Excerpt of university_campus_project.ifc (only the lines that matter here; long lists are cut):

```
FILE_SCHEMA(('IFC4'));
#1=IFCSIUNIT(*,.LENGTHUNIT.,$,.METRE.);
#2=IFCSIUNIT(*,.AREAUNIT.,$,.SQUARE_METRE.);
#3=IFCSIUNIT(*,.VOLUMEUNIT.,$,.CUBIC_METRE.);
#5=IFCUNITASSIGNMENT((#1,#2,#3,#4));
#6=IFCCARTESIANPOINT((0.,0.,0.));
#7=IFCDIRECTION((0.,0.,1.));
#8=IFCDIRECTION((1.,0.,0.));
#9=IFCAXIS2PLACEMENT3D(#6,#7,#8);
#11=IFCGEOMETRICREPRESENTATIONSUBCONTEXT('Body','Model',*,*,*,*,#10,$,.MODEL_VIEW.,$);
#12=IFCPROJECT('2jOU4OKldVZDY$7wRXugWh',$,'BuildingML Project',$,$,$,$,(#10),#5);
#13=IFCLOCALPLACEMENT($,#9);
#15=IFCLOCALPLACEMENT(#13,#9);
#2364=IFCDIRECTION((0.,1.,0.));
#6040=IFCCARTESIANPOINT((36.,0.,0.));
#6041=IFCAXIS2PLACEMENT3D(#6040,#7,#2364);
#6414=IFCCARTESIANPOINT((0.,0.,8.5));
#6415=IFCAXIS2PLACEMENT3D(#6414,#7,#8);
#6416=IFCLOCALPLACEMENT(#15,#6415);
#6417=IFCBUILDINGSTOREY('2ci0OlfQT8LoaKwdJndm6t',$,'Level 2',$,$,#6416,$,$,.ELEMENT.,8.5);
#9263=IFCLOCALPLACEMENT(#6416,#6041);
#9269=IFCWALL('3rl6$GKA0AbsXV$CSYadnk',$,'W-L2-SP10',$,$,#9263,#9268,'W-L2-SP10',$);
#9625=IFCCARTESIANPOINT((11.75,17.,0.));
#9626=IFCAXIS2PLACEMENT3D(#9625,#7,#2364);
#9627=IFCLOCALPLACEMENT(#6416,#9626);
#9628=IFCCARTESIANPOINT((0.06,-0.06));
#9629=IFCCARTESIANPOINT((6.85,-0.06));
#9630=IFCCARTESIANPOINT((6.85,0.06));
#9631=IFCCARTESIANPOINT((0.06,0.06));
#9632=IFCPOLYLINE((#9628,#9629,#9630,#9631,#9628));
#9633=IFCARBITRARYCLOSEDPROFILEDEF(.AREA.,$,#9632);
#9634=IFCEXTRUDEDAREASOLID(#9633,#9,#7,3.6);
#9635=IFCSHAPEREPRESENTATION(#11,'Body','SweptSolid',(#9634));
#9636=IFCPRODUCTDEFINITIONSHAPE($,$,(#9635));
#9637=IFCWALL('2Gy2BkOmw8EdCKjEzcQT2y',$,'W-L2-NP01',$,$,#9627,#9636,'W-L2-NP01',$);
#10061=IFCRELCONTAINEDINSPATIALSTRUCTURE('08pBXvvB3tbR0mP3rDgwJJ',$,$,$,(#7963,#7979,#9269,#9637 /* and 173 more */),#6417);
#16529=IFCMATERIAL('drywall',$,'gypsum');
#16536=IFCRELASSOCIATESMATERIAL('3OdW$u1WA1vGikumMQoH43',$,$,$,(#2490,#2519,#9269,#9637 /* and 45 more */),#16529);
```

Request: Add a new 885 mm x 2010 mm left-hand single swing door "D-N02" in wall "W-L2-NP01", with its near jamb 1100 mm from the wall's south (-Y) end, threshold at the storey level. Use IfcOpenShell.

```python
import numpy as np
import ifcopenshell
import ifcopenshell.api.feature
import ifcopenshell.api.geometry
import ifcopenshell.api.root
import ifcopenshell.api.spatial
import ifcopenshell.geom
import ifcopenshell.util.element
import ifcopenshell.util.placement
import ifcopenshell.util.representation
import ifcopenshell.util.shape
import ifcopenshell.util.unit

model = ifcopenshell.open("university_campus_project.ifc")
unit_scale = ifcopenshell.util.unit.calculate_unit_scale(model)
settings = ifcopenshell.geom.settings()


def volume(element):
    """Net volume in cubic metres, openings subtracted."""
    shape = ifcopenshell.geom.create_shape(settings, element)
    return ifcopenshell.util.shape.get_volume(shape.geometry)


wall = model.by_id(9637)
storey = ifcopenshell.util.element.get_container(wall, ifc_class="IfcBuildingStorey")
context = ifcopenshell.util.representation.get_context(model, "Model", "Body", "MODEL_VIEW")
before = volume(wall)

width, height, from_end, sill = 0.885, 2.01, 1.1, 0.0  # metres

# The wall runs along its own X axis, and the end named is its -X end.
wall_shape = ifcopenshell.geom.create_shape(settings, wall)
x, y, z = ifcopenshell.util.shape.get_vertices(wall_shape.geometry).T
start = x.min() + from_end
face, thickness = float(y.min()), float(y.max() - y.min())
wall_matrix = ifcopenshell.util.placement.get_local_placement(wall.ObjectPlacement)
level = ifcopenshell.util.placement.get_local_placement(storey.ObjectPlacement)[2, 3]


def in_wall(x, y):
    """Placement at x, y metres in the wall's axes, at sill height."""
    matrix = wall_matrix.copy()
    matrix[:, 3] = wall_matrix @ np.array([x / unit_scale, y / unit_scale, 0.0, 1.0])
    matrix[2, 3] = level + sill / unit_scale
    return matrix


# Opening: a box that overshoots both wall faces by 50 mm.
opening = ifcopenshell.api.root.create_entity(model, ifc_class="IfcOpeningElement", predefined_type="OPENING")
box = ifcopenshell.api.geometry.add_wall_representation(
    model, context=context, length=width, height=height, thickness=thickness + 0.1
)
ifcopenshell.api.geometry.assign_representation(model, product=opening, representation=box)
ifcopenshell.api.geometry.edit_object_placement(model, product=opening, matrix=in_wall(start, face - 0.05), is_si=False)
ifcopenshell.api.feature.add_feature(model, feature=opening, element=wall)

door = ifcopenshell.api.root.create_entity(model, ifc_class="IfcDoor", name="D-N02", predefined_type="DOOR")
door.OverallWidth, door.OverallHeight = width / unit_scale, height / unit_scale
door.OperationType = "SINGLE_SWING_LEFT"
body = ifcopenshell.api.geometry.add_door_representation(
    model,
    context=context,
    overall_width=door.OverallWidth,
    overall_height=door.OverallHeight,
    operation_type="SINGLE_SWING_LEFT",
    lining_properties={"LiningDepth": thickness / unit_scale, "ThresholdDepth": thickness / unit_scale},
)
ifcopenshell.api.geometry.assign_representation(model, product=door, representation=body)
ifcopenshell.api.spatial.assign_container(model, products=[door], relating_structure=storey)
ifcopenshell.api.feature.add_filling(model, opening=opening, element=door)

# The lining spans the wall, so the door starts at the wall face.
ifcopenshell.api.geometry.edit_object_placement(model, product=door, matrix=in_wall(start, face), is_si=False)

after = volume(wall)

print(f"wall volume {before:.3f} -> {after:.3f} m3")

model.write("university_campus_project_updated.ifc")
```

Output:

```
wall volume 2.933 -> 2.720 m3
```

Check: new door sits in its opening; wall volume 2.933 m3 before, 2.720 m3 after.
